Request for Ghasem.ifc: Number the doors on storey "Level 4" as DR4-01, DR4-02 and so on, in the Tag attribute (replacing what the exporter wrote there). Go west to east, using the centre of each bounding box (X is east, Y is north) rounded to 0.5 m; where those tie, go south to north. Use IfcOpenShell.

First a look at what the model holds.

```python
import ifcopenshell
import ifcopenshell.util.element
import ifcopenshell.util.placement

model = ifcopenshell.open("Ghasem.ifc")
print(model.schema)
storey = next(s for s in model.by_type("IfcBuildingStorey") if s.Name == "Level 4")
doors = [e for e in ifcopenshell.util.element.get_decomposition(storey) if e.is_a("IfcDoor")]
for e in sorted(doors, key=lambda e: e.id()):
    origin = ifcopenshell.util.placement.get_local_placement(e.ObjectPlacement)[:3, 3]
    print(e.id(), e.Tag, e.Name, origin.round(2) + 0.0, sep=" | ")
```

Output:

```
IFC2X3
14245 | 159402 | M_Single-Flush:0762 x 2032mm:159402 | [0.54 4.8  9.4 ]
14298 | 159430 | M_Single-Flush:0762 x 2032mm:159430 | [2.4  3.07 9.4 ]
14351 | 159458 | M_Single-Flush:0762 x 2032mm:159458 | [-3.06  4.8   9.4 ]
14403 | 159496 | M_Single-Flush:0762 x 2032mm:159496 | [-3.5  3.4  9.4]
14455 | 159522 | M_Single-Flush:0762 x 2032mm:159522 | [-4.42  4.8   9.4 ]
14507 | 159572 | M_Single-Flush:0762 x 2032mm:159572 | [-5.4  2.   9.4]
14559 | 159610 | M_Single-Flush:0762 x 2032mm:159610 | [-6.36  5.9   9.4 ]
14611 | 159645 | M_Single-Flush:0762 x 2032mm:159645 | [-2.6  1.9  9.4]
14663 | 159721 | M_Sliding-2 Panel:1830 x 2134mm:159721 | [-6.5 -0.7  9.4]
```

```python
import ifcopenshell
import ifcopenshell.geom
import ifcopenshell.util.element
import ifcopenshell.util.shape

model = ifcopenshell.open("Ghasem.ifc")
settings = ifcopenshell.geom.settings()
settings.set("use-world-coords", True)


def centre(element):
    shape = ifcopenshell.geom.create_shape(settings, element)
    return ifcopenshell.util.shape.get_bbox_centroid(shape.geometry)


storey = next(s for s in model.by_type("IfcBuildingStorey") if s.Name == "Level 4")
doors = [e for e in ifcopenshell.util.element.get_decomposition(storey) if e.is_a("IfcDoor")]

# Insertion points can sit at a corner or the storey origin, so sort by the geometry (in metres).
centres = {e: centre(e) for e in doors}
doors.sort(key=lambda e: (round(centres[e][0] / 0.5), centres[e][1]))

for i, e in enumerate(doors, start=1):
    number = f"DR4-{i:02d}"
    e.Tag = number
    print(e.id(), number)

model.write("Ghasem_updated.ifc")
```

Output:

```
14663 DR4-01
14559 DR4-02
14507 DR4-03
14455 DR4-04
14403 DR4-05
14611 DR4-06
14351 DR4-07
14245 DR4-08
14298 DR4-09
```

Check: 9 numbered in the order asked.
